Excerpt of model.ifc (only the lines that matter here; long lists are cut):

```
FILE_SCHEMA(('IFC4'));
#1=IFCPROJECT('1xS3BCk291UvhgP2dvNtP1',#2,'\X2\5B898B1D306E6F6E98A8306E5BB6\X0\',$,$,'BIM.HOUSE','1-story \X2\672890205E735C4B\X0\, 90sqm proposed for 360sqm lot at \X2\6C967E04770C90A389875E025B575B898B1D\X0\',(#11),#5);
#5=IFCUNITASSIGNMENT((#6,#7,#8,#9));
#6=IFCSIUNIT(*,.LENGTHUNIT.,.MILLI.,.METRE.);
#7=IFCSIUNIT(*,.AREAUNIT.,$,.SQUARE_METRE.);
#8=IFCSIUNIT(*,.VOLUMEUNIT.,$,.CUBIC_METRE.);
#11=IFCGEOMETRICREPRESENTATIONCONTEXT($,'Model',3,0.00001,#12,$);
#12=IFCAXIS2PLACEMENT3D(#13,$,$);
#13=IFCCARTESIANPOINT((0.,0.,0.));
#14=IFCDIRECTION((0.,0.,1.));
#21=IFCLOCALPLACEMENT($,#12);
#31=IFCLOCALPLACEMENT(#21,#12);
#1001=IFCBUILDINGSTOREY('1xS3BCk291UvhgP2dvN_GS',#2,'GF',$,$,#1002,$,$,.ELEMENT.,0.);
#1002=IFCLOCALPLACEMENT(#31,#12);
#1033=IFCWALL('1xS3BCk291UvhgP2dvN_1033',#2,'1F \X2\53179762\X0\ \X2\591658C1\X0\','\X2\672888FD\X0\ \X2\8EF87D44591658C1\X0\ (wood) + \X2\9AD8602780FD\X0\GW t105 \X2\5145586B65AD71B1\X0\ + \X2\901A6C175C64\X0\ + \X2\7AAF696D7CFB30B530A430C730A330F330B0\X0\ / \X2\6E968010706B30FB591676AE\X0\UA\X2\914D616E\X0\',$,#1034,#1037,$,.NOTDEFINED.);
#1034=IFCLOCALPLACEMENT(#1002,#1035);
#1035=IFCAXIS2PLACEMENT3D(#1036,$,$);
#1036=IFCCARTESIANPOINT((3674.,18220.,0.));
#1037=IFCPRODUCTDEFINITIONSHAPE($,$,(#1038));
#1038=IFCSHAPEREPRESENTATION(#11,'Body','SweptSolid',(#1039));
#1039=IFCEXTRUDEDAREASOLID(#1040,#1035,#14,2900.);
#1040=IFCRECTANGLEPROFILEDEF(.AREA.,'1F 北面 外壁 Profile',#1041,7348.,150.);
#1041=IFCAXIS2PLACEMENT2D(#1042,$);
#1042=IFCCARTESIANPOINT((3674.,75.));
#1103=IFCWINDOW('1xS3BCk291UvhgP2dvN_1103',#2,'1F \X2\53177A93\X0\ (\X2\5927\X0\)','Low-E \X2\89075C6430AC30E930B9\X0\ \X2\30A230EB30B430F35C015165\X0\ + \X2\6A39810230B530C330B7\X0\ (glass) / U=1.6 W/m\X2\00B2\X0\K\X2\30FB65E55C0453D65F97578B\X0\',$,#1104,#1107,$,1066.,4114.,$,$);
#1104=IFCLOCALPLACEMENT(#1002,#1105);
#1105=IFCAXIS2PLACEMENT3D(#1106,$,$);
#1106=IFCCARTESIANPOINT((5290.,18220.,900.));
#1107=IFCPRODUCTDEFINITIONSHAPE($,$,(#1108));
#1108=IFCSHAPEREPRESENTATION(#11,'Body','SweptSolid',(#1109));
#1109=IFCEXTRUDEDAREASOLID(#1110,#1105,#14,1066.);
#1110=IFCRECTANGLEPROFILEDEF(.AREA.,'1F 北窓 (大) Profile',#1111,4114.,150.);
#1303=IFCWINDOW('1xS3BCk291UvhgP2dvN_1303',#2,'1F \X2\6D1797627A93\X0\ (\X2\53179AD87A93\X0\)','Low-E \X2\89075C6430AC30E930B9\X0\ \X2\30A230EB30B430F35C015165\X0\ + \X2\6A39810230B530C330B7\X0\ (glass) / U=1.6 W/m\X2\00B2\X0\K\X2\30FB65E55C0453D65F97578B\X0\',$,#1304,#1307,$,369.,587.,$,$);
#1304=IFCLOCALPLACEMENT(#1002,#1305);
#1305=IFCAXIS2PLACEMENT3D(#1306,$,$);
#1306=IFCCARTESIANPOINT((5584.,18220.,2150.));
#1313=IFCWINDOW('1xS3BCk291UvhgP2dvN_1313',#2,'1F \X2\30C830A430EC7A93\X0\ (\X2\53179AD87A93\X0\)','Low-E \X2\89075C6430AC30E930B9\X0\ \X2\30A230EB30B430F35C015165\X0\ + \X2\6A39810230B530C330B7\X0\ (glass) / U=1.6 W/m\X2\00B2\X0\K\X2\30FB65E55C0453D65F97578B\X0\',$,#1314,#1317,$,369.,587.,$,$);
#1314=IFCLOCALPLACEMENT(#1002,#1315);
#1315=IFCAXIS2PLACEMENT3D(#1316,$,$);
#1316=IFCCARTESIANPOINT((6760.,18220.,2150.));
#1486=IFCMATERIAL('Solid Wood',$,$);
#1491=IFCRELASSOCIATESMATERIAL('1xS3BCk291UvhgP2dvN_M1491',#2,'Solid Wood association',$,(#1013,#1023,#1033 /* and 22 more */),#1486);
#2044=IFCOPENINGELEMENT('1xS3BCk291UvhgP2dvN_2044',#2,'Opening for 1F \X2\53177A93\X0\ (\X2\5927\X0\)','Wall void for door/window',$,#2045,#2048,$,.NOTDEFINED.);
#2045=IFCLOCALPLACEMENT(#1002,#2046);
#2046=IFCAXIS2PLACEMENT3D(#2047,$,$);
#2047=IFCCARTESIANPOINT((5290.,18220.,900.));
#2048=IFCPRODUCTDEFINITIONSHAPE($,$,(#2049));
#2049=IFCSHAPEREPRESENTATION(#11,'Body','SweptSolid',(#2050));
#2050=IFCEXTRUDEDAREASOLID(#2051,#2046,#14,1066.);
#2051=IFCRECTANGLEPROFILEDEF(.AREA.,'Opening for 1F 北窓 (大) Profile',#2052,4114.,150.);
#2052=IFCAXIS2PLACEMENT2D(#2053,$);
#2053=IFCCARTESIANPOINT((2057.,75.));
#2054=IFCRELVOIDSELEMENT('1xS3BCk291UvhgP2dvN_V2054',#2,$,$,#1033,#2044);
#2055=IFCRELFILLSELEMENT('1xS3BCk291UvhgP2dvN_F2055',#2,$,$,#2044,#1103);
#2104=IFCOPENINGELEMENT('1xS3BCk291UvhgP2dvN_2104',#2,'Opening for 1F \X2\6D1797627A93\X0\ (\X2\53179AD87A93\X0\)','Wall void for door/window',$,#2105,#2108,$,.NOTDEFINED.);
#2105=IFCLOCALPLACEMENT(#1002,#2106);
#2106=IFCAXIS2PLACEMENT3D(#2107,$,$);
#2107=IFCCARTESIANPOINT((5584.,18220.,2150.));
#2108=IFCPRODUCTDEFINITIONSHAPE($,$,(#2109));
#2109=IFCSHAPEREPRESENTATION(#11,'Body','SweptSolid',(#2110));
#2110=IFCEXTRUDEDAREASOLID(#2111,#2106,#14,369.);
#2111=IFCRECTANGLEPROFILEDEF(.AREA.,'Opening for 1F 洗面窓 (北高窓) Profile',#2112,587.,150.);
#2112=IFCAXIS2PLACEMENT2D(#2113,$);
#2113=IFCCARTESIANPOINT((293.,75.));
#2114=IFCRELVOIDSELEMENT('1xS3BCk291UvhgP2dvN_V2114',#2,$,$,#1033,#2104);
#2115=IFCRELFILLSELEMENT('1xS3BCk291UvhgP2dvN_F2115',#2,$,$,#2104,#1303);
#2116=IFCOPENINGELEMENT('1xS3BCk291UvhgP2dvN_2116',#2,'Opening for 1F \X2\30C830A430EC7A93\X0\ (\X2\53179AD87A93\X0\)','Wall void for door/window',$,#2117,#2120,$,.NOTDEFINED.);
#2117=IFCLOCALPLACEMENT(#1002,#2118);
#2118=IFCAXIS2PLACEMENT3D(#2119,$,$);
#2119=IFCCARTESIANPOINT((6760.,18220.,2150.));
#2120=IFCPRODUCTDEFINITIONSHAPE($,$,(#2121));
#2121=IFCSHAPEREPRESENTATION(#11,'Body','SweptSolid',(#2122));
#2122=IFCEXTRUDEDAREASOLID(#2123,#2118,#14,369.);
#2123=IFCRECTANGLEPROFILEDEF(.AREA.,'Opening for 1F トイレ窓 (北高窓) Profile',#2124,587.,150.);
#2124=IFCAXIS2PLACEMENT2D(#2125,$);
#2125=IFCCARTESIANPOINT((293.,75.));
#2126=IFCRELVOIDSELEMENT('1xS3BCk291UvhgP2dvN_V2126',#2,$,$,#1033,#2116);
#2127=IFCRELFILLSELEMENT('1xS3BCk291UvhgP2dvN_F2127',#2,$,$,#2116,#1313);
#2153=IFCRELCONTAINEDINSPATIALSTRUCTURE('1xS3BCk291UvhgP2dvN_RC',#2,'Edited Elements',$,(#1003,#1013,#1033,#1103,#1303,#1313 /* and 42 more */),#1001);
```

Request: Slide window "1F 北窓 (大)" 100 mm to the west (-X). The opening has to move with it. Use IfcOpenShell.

```python
import ifcopenshell
import ifcopenshell.api.geometry
import ifcopenshell.util.placement
import ifcopenshell.util.unit

model = ifcopenshell.open("model.ifc")
unit_scale = ifcopenshell.util.unit.calculate_unit_scale(model)

window = model.by_guid("1xS3BCk291UvhgP2dvN_1103")
opening = window.FillsVoids[0].RelatingOpeningElement
wall = opening.VoidsElements[0].RelatingBuildingElement

wall_matrix = ifcopenshell.util.placement.get_local_placement(wall.ObjectPlacement)
shift = wall_matrix[:3, 0] * -0.1 / unit_scale
before = ifcopenshell.util.placement.get_local_placement(window.ObjectPlacement)[:3, 3].copy()

# The window is not placed relative to its opening, so move both.
for product in (opening, window):
    matrix = ifcopenshell.util.placement.get_local_placement(product.ObjectPlacement)
    matrix[:3, 3] += shift
    ifcopenshell.api.geometry.edit_object_placement(model, product=product, matrix=matrix, is_si=False)

after = ifcopenshell.util.placement.get_local_placement(window.ObjectPlacement)[:3, 3]
print("window moved by", (after - before).round(3) + 0.0)

model.write("model_updated.ifc")
```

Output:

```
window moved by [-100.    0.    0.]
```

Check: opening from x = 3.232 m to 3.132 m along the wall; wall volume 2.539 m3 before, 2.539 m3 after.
